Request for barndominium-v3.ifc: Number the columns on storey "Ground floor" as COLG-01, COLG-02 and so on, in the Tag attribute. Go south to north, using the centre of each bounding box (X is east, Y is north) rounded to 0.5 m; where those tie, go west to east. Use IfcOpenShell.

First a look at what the model holds.

```python
import ifcopenshell
import ifcopenshell.util.element
import ifcopenshell.util.placement

model = ifcopenshell.open("barndominium-v3.ifc")
print(model.schema)
storey = next(s for s in model.by_type("IfcBuildingStorey") if s.Name == "Ground floor")
columns = [e for e in ifcopenshell.util.element.get_decomposition(storey) if e.is_a("IfcColumn")]
for e in sorted(columns, key=lambda e: e.id()):
    origin = ifcopenshell.util.placement.get_local_placement(e.ObjectPlacement)[:3, 3]
    print(e.id(), e.Tag, e.Name, origin.round(2) + 0.0, sep=" | ")
```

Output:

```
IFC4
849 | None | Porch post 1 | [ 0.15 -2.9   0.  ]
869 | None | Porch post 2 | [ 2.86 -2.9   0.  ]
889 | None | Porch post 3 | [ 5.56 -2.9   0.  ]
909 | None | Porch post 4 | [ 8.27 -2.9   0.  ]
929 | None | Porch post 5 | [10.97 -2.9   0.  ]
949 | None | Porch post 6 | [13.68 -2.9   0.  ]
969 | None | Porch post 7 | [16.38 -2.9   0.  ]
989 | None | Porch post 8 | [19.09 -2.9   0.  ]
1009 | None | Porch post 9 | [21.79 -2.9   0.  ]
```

```python
import ifcopenshell
import ifcopenshell.geom
import ifcopenshell.util.element
import ifcopenshell.util.shape

model = ifcopenshell.open("barndominium-v3.ifc")
settings = ifcopenshell.geom.settings()
settings.set("use-world-coords", True)


def centre(element):
    shape = ifcopenshell.geom.create_shape(settings, element)
    return ifcopenshell.util.shape.get_bbox_centroid(shape.geometry)


storey = next(s for s in model.by_type("IfcBuildingStorey") if s.Name == "Ground floor")
columns = [e for e in ifcopenshell.util.element.get_decomposition(storey) if e.is_a("IfcColumn")]

# Insertion points can sit at a corner or the storey origin, so sort by the geometry (in metres).
centres = {e: centre(e) for e in columns}
columns.sort(key=lambda e: (round(centres[e][1] / 0.5), centres[e][0]))

for i, e in enumerate(columns, start=1):
    number = f"COLG-{i:02d}"
    e.Tag = number
    print(e.id(), number)

model.write("barndominium-v3-out.ifc")
```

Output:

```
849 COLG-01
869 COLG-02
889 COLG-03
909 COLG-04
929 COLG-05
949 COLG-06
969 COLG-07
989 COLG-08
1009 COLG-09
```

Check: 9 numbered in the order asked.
